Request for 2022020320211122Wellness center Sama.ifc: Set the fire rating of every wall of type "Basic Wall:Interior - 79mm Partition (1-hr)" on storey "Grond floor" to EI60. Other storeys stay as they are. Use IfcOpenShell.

First a look at what the model holds.

```python
import ifcopenshell
import ifcopenshell.util.element

model = ifcopenshell.open("2022020320211122Wellness center Sama.ifc")
print(model.schema)
storey = next(s for s in model.by_type("IfcBuildingStorey") if s.Name == "Grond floor")
walls = [e for e in ifcopenshell.util.element.get_decomposition(storey) if e.is_a("IfcWall")]
seen = {}
for e in walls:
    element_type = ifcopenshell.util.element.get_type(e)
    key = (element_type.Name if element_type != e and element_type else None, ifcopenshell.util.element.get_pset(e, "Pset_WallCommon", "FireRating"))
    seen[key] = seen.get(key, 0) + 1
for (name, value), count in sorted(seen.items(), key=str):
    print(count, "x", name, "|", value)
```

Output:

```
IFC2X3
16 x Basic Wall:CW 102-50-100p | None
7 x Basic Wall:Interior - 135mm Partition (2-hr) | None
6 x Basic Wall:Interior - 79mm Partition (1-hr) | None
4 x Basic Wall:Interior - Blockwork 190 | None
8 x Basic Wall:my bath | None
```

```python
import ifcopenshell
import ifcopenshell.api.pset
import ifcopenshell.util.element

model = ifcopenshell.open("2022020320211122Wellness center Sama.ifc")

storey = next(s for s in model.by_type("IfcBuildingStorey") if s.Name == "Grond floor")
walls = [e for e in ifcopenshell.util.element.get_decomposition(storey) if e.is_a("IfcWall")]

count = 0
for e in walls:
    element_type = ifcopenshell.util.element.get_type(e)
    if element_type in (None, e) or element_type.Name != "Basic Wall:Interior - 79mm Partition (1-hr)":
        continue
    # add_pset returns the element's existing set when there is one.
    pset = ifcopenshell.api.pset.add_pset(model, product=e, name="Pset_WallCommon")
    ifcopenshell.api.pset.edit_pset(model, pset=pset, properties={"FireRating": "EI60"})
    count += 1

print(count, "walls updated")

model.write("2022020320211122Wellness center Sama_edited.ifc")
```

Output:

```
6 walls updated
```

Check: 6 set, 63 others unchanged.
